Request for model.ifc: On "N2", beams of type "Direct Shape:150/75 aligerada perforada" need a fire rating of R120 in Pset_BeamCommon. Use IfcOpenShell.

First a look at what the model holds.

```python
import ifcopenshell
import ifcopenshell.util.element

model = ifcopenshell.open("model.ifc")
print(model.schema)
storey = next(s for s in model.by_type("IfcBuildingStorey") if s.Name == "N2")
beams = [e for e in ifcopenshell.util.element.get_decomposition(storey) if e.is_a("IfcBeam")]
seen = {}
for e in beams:
    element_type = ifcopenshell.util.element.get_type(e)
    key = (element_type.Name if element_type != e and element_type else None, ifcopenshell.util.element.get_pset(e, "Pset_BeamCommon", "FireRating"))
    seen[key] = seen.get(key, 0) + 1
for (name, value), count in sorted(seen.items(), key=str):
    print(count, "x", name, "|", value)
```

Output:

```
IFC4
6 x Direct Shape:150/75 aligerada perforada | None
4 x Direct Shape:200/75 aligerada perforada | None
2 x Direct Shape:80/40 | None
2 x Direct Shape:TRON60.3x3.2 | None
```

```python
import ifcopenshell
import ifcopenshell.api.pset
import ifcopenshell.util.element

model = ifcopenshell.open("model.ifc")

storey = next(s for s in model.by_type("IfcBuildingStorey") if s.Name == "N2")
beams = [e for e in ifcopenshell.util.element.get_decomposition(storey) if e.is_a("IfcBeam")]

count = 0
for e in beams:
    element_type = ifcopenshell.util.element.get_type(e)
    if element_type in (None, e) or element_type.Name != "Direct Shape:150/75 aligerada perforada":
        continue
    # add_pset returns the element's existing set when there is one.
    pset = ifcopenshell.api.pset.add_pset(model, product=e, name="Pset_BeamCommon")
    ifcopenshell.api.pset.edit_pset(model, pset=pset, properties={"FireRating": "R120"})
    count += 1

print(count, "beams updated")

model.write("model_v2.ifc")
```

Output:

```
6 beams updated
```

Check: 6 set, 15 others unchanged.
